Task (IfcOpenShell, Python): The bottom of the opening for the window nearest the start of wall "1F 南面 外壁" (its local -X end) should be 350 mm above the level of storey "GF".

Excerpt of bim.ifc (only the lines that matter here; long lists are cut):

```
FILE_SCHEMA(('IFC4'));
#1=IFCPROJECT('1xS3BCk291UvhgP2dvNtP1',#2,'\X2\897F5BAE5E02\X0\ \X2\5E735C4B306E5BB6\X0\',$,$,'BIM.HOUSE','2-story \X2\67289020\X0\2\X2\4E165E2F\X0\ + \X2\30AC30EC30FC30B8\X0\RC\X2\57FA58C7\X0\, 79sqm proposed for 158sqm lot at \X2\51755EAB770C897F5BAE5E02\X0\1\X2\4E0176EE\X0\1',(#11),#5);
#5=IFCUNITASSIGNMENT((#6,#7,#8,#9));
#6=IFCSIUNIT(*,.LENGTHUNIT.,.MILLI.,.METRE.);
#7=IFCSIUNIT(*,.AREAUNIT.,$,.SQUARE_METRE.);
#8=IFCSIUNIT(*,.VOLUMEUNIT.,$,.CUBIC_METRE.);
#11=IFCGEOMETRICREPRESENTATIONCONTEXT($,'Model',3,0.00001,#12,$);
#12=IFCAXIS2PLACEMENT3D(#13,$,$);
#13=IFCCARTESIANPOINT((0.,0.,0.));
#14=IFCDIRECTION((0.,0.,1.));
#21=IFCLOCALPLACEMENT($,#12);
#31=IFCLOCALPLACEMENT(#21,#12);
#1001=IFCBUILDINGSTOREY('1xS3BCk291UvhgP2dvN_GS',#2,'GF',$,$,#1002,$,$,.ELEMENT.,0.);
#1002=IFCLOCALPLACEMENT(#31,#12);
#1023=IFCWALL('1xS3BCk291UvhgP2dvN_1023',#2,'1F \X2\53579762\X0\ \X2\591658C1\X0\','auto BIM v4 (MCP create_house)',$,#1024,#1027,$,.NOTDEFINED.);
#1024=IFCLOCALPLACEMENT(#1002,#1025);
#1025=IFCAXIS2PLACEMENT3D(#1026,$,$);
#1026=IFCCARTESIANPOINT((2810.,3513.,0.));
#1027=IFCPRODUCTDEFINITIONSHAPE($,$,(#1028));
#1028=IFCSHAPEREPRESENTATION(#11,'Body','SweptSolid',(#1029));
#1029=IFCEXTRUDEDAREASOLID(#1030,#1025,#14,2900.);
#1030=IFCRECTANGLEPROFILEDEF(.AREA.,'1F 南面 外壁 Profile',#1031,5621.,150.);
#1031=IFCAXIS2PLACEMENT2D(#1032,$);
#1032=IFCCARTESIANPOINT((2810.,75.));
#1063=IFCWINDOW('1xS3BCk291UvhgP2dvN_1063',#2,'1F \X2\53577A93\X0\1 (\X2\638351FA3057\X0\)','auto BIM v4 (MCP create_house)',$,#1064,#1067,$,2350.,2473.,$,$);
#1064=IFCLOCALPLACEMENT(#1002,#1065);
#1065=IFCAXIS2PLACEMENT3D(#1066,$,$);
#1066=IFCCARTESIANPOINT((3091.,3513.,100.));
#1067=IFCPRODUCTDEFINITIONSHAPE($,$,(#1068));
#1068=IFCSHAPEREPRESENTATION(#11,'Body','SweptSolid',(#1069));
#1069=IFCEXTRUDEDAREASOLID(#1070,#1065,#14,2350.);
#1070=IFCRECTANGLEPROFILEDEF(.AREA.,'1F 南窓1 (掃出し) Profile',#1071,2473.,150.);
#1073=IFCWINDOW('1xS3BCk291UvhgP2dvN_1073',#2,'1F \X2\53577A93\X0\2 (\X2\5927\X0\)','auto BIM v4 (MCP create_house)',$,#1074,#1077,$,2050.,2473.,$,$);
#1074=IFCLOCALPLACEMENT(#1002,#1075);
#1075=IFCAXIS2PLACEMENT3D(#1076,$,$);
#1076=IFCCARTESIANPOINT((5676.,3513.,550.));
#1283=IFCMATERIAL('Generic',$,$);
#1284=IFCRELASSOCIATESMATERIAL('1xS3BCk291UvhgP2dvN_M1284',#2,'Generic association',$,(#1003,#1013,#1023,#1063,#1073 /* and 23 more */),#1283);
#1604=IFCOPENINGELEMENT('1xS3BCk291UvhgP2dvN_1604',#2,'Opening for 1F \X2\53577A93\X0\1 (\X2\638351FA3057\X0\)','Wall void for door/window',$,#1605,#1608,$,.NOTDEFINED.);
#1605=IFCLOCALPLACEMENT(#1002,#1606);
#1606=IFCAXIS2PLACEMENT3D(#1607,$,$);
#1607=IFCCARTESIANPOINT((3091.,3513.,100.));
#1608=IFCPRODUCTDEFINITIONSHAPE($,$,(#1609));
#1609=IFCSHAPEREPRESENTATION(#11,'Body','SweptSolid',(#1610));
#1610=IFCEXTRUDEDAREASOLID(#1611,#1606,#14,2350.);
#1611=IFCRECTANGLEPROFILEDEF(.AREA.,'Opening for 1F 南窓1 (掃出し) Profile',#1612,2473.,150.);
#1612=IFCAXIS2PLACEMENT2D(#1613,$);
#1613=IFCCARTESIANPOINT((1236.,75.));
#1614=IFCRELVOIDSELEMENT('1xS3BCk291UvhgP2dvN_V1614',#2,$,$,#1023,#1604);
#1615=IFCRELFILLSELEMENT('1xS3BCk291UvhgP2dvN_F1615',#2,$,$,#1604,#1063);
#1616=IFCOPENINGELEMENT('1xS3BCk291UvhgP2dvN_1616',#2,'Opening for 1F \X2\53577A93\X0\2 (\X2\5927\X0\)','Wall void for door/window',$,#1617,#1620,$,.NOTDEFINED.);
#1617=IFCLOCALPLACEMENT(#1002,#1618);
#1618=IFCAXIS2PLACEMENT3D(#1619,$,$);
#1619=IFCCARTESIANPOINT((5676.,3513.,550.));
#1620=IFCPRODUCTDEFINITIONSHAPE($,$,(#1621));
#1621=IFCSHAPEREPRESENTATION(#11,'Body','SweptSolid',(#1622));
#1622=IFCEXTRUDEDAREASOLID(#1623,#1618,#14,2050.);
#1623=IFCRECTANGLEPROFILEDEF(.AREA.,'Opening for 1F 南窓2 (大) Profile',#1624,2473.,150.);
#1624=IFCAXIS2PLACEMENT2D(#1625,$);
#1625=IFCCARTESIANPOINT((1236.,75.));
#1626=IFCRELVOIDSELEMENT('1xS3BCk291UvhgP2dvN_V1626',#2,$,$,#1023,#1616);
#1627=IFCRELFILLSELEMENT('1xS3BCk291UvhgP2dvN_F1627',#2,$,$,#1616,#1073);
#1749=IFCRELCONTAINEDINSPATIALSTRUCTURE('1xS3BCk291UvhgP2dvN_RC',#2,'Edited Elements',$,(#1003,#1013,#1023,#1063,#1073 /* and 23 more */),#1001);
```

```python
import numpy as np
import ifcopenshell
import ifcopenshell.api.geometry
import ifcopenshell.geom
import ifcopenshell.util.element
import ifcopenshell.util.placement
import ifcopenshell.util.shape
import ifcopenshell.util.unit

model = ifcopenshell.open("bim.ifc")
unit_scale = ifcopenshell.util.unit.calculate_unit_scale(model)

window = model.by_guid("1xS3BCk291UvhgP2dvN_1063")
opening = window.FillsVoids[0].RelatingOpeningElement
storey = ifcopenshell.util.element.get_container(window, ifc_class="IfcBuildingStorey")
level = ifcopenshell.util.placement.get_local_placement(storey.ObjectPlacement)[2, 3]

# The opening's origin need not be at the sill, so measure its lowest point.
shape = ifcopenshell.geom.create_shape(ifcopenshell.geom.settings(), opening)
bottom = ifcopenshell.util.shape.get_shape_bottom_elevation(shape, shape.geometry) / unit_scale
dz = level + 350.0 - bottom

shift = np.array([0.0, 0.0, dz])
# The window is not placed relative to its opening, so move both.
for product in (opening, window):
    matrix = ifcopenshell.util.placement.get_local_placement(product.ObjectPlacement)
    matrix[:3, 3] += shift
    ifcopenshell.api.geometry.edit_object_placement(model, product=product, matrix=matrix, is_si=False)

print(f"moved by {dz * unit_scale:+.3f} m")

model.write("bim_updated.ifc")
```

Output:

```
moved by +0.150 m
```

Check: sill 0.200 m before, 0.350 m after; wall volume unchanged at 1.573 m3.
